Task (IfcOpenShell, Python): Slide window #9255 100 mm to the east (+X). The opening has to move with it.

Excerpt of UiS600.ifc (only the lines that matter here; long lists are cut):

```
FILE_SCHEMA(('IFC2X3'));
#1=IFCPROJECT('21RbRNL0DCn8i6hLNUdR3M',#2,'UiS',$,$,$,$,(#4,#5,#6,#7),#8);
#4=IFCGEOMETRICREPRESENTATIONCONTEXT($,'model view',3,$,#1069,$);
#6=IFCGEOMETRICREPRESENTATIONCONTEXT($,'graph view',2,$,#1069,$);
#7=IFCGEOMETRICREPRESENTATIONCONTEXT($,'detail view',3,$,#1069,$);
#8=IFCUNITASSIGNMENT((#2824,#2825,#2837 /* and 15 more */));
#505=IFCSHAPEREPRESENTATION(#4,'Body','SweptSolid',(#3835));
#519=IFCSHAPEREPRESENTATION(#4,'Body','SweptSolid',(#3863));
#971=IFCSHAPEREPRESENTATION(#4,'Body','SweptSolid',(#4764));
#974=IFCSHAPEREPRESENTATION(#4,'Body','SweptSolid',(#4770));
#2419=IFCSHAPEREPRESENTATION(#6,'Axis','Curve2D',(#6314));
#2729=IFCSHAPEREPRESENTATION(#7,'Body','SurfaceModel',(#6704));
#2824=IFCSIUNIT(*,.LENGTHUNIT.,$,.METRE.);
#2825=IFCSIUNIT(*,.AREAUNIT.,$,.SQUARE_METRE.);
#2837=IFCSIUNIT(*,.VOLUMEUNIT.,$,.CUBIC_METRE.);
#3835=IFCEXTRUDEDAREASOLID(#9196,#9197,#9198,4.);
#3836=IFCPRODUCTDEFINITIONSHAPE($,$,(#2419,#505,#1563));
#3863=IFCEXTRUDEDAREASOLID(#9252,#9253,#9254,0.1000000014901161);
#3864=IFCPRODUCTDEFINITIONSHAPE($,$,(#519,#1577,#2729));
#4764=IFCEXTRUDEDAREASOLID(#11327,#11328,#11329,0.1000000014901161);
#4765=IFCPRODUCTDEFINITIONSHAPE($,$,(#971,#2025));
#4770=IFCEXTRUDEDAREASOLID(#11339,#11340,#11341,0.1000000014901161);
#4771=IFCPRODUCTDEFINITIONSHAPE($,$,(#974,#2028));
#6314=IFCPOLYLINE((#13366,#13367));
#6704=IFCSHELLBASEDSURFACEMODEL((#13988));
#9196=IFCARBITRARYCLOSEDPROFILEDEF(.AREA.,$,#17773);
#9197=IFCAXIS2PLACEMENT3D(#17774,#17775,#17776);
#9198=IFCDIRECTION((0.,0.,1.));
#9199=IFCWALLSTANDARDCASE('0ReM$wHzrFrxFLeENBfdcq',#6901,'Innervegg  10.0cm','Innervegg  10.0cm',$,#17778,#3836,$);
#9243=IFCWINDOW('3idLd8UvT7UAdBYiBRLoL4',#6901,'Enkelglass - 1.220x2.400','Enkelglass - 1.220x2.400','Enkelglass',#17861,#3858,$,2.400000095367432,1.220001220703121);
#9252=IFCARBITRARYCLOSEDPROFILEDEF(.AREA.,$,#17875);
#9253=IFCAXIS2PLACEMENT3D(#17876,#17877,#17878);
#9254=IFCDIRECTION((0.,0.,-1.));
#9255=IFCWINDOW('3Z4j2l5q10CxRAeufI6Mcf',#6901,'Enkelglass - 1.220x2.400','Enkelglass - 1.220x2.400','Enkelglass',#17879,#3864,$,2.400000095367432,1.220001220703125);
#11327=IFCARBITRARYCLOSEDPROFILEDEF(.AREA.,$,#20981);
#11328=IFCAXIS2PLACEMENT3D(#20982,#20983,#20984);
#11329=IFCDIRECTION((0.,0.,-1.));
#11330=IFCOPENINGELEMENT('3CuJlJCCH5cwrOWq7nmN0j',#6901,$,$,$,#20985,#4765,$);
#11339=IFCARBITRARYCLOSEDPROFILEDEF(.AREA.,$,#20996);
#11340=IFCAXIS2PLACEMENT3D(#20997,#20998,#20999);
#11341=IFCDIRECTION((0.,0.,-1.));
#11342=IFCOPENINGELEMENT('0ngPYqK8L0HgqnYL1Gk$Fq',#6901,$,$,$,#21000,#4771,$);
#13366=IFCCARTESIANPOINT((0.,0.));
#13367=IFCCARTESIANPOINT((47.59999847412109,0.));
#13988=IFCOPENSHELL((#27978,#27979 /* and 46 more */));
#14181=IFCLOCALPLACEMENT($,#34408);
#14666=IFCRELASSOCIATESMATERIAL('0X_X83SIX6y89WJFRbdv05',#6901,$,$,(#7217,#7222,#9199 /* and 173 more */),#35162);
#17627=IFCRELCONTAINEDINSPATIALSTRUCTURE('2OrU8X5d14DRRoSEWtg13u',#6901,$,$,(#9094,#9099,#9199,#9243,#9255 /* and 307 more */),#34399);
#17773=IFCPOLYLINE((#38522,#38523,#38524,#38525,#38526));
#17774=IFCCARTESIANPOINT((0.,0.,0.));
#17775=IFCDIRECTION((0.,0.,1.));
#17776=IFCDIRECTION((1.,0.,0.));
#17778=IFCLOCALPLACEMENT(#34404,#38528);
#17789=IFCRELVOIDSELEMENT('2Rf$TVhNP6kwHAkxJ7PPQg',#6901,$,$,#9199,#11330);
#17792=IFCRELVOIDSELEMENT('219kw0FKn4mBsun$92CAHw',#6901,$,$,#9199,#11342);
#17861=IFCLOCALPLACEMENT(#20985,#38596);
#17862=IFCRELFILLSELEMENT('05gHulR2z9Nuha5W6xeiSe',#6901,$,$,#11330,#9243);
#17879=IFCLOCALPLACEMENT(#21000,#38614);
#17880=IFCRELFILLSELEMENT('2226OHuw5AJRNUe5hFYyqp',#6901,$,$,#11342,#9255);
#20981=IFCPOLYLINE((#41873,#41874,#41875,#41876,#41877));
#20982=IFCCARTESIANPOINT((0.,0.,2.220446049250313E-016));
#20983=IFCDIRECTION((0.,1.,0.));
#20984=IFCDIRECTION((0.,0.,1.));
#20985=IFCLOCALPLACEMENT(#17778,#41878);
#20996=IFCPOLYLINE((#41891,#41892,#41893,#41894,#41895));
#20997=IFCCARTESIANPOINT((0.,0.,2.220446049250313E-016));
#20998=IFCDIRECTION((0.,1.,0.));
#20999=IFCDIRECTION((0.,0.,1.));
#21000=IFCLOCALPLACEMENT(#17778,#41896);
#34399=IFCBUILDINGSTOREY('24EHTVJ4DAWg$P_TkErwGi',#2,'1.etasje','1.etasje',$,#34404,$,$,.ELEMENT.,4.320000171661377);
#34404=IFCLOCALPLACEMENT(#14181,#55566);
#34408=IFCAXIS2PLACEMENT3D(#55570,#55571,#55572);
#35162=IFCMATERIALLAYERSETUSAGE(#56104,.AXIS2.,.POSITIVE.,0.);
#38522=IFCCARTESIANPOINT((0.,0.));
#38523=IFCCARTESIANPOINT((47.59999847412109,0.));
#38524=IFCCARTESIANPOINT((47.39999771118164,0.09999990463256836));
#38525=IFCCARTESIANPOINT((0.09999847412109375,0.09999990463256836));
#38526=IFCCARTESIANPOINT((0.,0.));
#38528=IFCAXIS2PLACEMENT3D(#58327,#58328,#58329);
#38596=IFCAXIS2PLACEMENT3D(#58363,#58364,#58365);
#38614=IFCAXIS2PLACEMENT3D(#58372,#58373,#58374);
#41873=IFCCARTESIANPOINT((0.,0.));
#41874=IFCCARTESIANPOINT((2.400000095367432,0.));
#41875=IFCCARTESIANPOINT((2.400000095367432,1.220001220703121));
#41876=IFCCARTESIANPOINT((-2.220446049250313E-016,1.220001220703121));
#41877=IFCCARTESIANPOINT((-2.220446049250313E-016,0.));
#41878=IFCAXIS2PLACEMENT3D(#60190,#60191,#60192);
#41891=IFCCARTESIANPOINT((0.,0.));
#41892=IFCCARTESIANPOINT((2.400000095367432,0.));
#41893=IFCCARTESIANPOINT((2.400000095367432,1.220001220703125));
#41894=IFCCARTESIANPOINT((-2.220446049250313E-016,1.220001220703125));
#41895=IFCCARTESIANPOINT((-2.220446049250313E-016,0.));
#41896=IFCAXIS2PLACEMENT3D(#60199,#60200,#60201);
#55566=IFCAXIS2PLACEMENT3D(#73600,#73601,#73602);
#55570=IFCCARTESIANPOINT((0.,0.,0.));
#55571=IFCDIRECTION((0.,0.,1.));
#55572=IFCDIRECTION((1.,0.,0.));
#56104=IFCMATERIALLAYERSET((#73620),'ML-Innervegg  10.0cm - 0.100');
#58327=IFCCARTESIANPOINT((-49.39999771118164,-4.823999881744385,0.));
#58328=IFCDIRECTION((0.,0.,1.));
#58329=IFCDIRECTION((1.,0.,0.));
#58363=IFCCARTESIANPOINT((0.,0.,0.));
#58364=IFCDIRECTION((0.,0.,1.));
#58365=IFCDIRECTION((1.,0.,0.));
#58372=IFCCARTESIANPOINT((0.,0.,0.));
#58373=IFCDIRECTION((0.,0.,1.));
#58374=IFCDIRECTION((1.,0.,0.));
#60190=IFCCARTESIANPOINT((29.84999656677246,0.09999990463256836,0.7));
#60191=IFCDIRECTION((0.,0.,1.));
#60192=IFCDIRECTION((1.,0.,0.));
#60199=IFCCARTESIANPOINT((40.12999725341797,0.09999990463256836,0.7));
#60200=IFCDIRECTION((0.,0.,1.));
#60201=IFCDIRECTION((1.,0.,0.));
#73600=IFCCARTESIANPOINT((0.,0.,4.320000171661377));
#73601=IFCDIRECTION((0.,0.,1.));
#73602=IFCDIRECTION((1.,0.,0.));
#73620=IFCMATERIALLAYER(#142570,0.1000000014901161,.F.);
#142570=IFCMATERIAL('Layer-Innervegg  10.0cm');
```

```python
import ifcopenshell
import ifcopenshell.api.geometry
import ifcopenshell.util.placement
import ifcopenshell.util.unit

model = ifcopenshell.open("UiS600.ifc")
unit_scale = ifcopenshell.util.unit.calculate_unit_scale(model)

window = model.by_guid("3Z4j2l5q10CxRAeufI6Mcf")
opening = window.FillsVoids[0].RelatingOpeningElement
wall = opening.VoidsElements[0].RelatingBuildingElement

wall_matrix = ifcopenshell.util.placement.get_local_placement(wall.ObjectPlacement)
shift = wall_matrix[:3, 0] * 0.1 / unit_scale
before = ifcopenshell.util.placement.get_local_placement(window.ObjectPlacement)[:3, 3].copy()

# The window is placed relative to its opening, so it follows when the opening moves.
matrix = ifcopenshell.util.placement.get_local_placement(opening.ObjectPlacement)
matrix[:3, 3] += shift
ifcopenshell.api.geometry.edit_object_placement(
    model, product=opening, matrix=matrix, is_si=False, should_transform_children=True
)

after = ifcopenshell.util.placement.get_local_placement(window.ObjectPlacement)[:3, 3]
print("window moved by", (after - before).round(3) + 0.0)

model.write("UiS600-out.ifc")
```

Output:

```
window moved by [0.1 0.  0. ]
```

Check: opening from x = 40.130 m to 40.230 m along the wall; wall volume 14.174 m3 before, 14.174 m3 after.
